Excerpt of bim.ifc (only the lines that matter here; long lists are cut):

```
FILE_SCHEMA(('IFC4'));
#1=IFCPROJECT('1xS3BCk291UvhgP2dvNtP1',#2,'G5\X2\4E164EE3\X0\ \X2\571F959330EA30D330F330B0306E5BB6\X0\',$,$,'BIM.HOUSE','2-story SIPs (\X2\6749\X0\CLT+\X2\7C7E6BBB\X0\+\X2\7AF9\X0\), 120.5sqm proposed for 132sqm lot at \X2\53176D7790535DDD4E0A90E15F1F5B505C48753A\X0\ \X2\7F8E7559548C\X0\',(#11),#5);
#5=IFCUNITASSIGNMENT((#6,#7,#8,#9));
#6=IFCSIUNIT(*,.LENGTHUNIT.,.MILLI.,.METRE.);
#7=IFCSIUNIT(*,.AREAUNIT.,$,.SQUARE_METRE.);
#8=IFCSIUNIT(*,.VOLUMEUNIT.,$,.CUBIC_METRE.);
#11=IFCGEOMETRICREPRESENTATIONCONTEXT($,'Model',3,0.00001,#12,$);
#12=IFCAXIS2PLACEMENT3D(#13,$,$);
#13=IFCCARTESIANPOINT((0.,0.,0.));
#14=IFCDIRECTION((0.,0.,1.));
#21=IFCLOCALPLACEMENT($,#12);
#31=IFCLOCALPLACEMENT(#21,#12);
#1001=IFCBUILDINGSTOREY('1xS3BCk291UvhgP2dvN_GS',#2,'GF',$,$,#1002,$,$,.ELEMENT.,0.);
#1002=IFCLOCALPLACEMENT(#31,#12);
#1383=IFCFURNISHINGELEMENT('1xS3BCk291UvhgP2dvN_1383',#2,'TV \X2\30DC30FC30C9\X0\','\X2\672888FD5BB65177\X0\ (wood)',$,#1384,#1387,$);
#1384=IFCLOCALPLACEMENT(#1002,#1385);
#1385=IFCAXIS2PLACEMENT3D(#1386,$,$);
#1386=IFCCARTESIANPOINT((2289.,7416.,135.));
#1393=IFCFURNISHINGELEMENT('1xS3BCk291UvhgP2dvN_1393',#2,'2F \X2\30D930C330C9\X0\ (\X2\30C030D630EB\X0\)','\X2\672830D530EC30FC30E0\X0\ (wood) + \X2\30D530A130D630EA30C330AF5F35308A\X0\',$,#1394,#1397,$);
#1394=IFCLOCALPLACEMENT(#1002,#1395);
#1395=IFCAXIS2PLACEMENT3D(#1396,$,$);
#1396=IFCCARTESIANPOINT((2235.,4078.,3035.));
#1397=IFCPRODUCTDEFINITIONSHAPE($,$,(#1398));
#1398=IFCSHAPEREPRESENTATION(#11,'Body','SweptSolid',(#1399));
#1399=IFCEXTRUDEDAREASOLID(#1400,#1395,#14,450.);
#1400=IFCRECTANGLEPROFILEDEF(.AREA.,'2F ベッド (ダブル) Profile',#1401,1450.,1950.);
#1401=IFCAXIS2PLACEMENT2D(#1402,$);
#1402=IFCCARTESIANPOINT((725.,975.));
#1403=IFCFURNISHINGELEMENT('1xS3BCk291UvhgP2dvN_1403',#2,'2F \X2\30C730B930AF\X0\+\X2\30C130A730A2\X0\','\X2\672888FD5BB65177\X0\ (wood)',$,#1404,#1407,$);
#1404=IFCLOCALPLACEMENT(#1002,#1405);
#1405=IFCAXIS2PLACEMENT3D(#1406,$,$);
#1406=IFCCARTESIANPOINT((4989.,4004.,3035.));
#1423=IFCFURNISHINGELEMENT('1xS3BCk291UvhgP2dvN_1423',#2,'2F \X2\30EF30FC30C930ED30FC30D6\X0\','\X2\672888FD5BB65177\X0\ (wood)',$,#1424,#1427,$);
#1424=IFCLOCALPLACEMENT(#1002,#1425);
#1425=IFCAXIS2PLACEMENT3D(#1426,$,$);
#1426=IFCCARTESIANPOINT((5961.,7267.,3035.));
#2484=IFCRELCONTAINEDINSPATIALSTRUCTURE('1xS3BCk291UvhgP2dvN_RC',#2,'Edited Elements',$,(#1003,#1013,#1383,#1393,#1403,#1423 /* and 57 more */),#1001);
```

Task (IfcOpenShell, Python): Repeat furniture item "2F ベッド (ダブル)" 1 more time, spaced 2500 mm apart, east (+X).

```python
import numpy as np
import ifcopenshell
import ifcopenshell.api.geometry
import ifcopenshell.api.root
import ifcopenshell.util.element
import ifcopenshell.util.placement
import ifcopenshell.util.unit

model = ifcopenshell.open("bim.ifc")
unit_scale = ifcopenshell.util.unit.calculate_unit_scale(model)


def reuse_history(source, copy):
    """copy_class also copies each property set's owner history, people and application; keep the originals."""
    for rel in copy.IsDefinedBy:
        if rel.is_a("IfcRelDefinesByProperties") and (history := rel.RelatingPropertyDefinition.OwnerHistory):
            rel.RelatingPropertyDefinition.OwnerHistory = source.OwnerHistory
            ifcopenshell.util.element.remove_deep2(model, history)


source = model.by_guid("1xS3BCk291UvhgP2dvN_1393")
base = ifcopenshell.util.placement.get_local_placement(source.ObjectPlacement)
step = np.array([1.0, 0.0, 0.0]) * 2.5 / unit_scale

for i in range(1, 2):
    copy = ifcopenshell.api.root.copy_class(model, product=source)
    copy.Representation = ifcopenshell.util.element.copy_deep(
        model, source.Representation, exclude=["IfcGeometricRepresentationContext", "IfcRepresentationMap"]
    )
    reuse_history(source, copy)
    matrix = base.copy()
    matrix[:3, 3] += i * step
    print("added at", matrix[:3, 3].round(3) + 0.0)
    ifcopenshell.api.geometry.edit_object_placement(model, product=copy, matrix=matrix, is_si=False)

model.write("bim_updated.ifc")
```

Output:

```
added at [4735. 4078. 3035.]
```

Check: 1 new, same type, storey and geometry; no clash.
